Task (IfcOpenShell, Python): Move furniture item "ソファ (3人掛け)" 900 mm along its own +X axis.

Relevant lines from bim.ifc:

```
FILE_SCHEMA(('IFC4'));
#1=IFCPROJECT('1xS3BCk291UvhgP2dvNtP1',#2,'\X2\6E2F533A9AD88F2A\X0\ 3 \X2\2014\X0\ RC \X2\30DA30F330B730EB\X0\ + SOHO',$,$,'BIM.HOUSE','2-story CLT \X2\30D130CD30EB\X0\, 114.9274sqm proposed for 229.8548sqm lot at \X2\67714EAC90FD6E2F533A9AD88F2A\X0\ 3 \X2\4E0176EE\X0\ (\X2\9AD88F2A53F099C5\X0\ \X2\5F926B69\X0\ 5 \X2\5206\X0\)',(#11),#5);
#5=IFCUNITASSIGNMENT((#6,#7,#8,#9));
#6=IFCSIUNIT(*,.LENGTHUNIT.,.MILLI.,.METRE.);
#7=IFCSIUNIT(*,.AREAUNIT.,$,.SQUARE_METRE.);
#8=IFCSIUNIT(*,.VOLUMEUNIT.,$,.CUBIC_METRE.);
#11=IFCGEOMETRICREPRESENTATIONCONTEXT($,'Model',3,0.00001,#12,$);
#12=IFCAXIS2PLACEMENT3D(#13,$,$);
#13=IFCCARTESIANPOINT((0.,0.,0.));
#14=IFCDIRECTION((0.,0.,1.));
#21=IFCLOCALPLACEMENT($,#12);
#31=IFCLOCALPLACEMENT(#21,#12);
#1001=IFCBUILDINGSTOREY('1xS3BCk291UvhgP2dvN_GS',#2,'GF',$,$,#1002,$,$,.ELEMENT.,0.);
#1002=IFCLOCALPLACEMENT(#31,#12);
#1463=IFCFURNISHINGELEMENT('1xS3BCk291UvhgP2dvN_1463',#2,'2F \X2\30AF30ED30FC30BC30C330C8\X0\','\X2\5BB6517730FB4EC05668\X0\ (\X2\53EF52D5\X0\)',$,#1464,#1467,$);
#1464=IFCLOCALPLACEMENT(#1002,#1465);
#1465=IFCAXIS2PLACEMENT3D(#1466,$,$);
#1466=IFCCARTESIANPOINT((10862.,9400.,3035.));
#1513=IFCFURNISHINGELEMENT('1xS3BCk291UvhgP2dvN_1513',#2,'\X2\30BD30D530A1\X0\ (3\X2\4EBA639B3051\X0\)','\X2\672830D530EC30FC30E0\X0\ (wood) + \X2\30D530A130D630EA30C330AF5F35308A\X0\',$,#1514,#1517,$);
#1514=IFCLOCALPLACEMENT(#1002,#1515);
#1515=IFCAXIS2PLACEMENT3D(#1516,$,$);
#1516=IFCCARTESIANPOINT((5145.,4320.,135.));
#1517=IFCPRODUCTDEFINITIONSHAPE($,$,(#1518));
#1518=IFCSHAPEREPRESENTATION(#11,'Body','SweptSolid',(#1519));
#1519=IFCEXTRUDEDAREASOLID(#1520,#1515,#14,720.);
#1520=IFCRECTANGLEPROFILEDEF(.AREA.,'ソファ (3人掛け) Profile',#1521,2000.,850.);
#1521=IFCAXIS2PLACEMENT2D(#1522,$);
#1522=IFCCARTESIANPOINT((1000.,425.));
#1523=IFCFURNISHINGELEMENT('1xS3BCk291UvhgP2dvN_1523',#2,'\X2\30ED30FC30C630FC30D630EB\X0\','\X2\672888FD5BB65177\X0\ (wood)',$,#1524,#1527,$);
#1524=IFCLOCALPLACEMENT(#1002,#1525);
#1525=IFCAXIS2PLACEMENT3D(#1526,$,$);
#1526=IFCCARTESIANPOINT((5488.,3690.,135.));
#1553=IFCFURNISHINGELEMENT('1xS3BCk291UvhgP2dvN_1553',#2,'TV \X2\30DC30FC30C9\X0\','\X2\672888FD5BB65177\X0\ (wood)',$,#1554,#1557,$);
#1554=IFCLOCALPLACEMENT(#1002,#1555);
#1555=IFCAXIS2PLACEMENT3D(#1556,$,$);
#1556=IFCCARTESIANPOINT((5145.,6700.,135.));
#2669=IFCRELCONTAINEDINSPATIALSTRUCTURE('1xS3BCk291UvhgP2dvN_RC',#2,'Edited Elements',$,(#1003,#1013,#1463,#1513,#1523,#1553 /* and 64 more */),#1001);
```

```python
import ifcopenshell
import ifcopenshell.api.geometry
import ifcopenshell.util.placement

model = ifcopenshell.open("bim.ifc")

item = model.by_id(1513)
matrix = ifcopenshell.util.placement.get_local_placement(item.ObjectPlacement)
matrix[:3, 3] += matrix[:3, 0] * 900.0
ifcopenshell.api.geometry.edit_object_placement(model, product=item, matrix=matrix, is_si=False)

print(ifcopenshell.util.placement.get_local_placement(item.ObjectPlacement).round(3) + 0.0)

model.write("bim_rev.ifc")
```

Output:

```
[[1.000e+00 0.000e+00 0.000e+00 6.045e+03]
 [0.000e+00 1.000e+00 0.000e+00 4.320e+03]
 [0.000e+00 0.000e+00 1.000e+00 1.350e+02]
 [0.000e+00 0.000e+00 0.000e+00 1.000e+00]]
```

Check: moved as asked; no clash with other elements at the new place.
